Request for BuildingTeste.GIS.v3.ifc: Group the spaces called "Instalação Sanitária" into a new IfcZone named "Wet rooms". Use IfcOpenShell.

First a look at what the model holds.

```python
import ifcopenshell

model = ifcopenshell.open("BuildingTeste.GIS.v3.ifc")
print(model.schema)
seen = {}
for space in model.by_type("IfcSpace"):
    seen[space.LongName] = seen.get(space.LongName, 0) + 1
for name, count in sorted(seen.items(), key=str):
    print(count, "x", name)
print("zones:", [z.Name for z in model.by_type("IfcZone")][:20])
```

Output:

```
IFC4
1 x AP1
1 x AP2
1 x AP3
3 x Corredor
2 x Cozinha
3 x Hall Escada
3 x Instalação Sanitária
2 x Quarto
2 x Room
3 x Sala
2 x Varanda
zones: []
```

```python
import ifcopenshell
import ifcopenshell.api.group
import ifcopenshell.api.root

model = ifcopenshell.open("BuildingTeste.GIS.v3.ifc")

names = {"Instalação Sanitária"}
spaces = [s for s in model.by_type("IfcSpace") if s.LongName in names]

zone = ifcopenshell.api.root.create_entity(model, ifc_class="IfcZone", name="Wet rooms")
ifcopenshell.api.group.assign_group(model, products=spaces, group=zone)
print(len(spaces), "spaces in", zone.Name)

model.write("BuildingTeste.GIS.v3_v2.ifc")
```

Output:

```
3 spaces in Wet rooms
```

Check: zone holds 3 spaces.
